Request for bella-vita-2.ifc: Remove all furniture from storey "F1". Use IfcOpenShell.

First a look at what the model holds.

```python
import ifcopenshell
import ifcopenshell.util.element

model = ifcopenshell.open("bella-vita-2.ifc")
print(model.schema)
storey = next(s for s in model.by_type("IfcBuildingStorey") if s.Name == "F1")
furniture = [e for e in ifcopenshell.util.element.get_decomposition(storey) if e.is_a("IfcFurnishingElement")]
seen = {}
for e in furniture:
    element_type = ifcopenshell.util.element.get_type(e)
    name = element_type.Name if element_type not in (None, e) else None
    seen[name] = seen.get(name, 0) + 1
for name, count in sorted(seen.items(), key=str):
    print(count, "x", name)
```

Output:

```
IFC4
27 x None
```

```python
import ifcopenshell
import ifcopenshell.api.root
import ifcopenshell.util.element

model = ifcopenshell.open("bella-vita-2.ifc")

storey = next(s for s in model.by_type("IfcBuildingStorey") if s.Name == "F1")
furniture = [e for e in ifcopenshell.util.element.get_decomposition(storey) if e.is_a("IfcFurnishingElement")]

for e in furniture:
    ifcopenshell.api.root.remove_product(model, product=e)
print(len(furniture), "removed")

model.write("bella-vita-2_rev.ifc")
```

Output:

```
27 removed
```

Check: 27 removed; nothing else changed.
